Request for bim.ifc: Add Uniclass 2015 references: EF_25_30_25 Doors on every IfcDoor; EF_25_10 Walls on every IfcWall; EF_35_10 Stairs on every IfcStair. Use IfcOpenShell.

First a look at what the model holds.

```python
import ifcopenshell

model = ifcopenshell.open("bim.ifc")
print(model.schema)
print("classifications:", [c.Name for c in model.by_type("IfcClassification")])
for ifc_class in ("IfcDoor", "IfcRoof", "IfcStair", "IfcWall", "IfcWindow"):
    print(ifc_class, len(model.by_type(ifc_class)))
```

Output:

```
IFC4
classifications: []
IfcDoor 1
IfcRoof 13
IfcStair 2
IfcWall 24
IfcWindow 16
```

```python
import ifcopenshell
import ifcopenshell.api.classification

model = ifcopenshell.open("bim.ifc")

system = ifcopenshell.api.classification.add_classification(model, classification="Uniclass 2015")

codes = {
    "IfcDoor": ("EF_25_30_25", "Doors"),
    "IfcWall": ("EF_25_10", "Walls"),
    "IfcStair": ("EF_35_10", "Stairs"),
}
for ifc_class, (code, name) in codes.items():
    products = model.by_type(ifc_class)
    ifcopenshell.api.classification.add_reference(
        model, products=products, classification=system, identification=code, name=name
    )
    print(code, len(products))

model.write("bim_edited.ifc")
```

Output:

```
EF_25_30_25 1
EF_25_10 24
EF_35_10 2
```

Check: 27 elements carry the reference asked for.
